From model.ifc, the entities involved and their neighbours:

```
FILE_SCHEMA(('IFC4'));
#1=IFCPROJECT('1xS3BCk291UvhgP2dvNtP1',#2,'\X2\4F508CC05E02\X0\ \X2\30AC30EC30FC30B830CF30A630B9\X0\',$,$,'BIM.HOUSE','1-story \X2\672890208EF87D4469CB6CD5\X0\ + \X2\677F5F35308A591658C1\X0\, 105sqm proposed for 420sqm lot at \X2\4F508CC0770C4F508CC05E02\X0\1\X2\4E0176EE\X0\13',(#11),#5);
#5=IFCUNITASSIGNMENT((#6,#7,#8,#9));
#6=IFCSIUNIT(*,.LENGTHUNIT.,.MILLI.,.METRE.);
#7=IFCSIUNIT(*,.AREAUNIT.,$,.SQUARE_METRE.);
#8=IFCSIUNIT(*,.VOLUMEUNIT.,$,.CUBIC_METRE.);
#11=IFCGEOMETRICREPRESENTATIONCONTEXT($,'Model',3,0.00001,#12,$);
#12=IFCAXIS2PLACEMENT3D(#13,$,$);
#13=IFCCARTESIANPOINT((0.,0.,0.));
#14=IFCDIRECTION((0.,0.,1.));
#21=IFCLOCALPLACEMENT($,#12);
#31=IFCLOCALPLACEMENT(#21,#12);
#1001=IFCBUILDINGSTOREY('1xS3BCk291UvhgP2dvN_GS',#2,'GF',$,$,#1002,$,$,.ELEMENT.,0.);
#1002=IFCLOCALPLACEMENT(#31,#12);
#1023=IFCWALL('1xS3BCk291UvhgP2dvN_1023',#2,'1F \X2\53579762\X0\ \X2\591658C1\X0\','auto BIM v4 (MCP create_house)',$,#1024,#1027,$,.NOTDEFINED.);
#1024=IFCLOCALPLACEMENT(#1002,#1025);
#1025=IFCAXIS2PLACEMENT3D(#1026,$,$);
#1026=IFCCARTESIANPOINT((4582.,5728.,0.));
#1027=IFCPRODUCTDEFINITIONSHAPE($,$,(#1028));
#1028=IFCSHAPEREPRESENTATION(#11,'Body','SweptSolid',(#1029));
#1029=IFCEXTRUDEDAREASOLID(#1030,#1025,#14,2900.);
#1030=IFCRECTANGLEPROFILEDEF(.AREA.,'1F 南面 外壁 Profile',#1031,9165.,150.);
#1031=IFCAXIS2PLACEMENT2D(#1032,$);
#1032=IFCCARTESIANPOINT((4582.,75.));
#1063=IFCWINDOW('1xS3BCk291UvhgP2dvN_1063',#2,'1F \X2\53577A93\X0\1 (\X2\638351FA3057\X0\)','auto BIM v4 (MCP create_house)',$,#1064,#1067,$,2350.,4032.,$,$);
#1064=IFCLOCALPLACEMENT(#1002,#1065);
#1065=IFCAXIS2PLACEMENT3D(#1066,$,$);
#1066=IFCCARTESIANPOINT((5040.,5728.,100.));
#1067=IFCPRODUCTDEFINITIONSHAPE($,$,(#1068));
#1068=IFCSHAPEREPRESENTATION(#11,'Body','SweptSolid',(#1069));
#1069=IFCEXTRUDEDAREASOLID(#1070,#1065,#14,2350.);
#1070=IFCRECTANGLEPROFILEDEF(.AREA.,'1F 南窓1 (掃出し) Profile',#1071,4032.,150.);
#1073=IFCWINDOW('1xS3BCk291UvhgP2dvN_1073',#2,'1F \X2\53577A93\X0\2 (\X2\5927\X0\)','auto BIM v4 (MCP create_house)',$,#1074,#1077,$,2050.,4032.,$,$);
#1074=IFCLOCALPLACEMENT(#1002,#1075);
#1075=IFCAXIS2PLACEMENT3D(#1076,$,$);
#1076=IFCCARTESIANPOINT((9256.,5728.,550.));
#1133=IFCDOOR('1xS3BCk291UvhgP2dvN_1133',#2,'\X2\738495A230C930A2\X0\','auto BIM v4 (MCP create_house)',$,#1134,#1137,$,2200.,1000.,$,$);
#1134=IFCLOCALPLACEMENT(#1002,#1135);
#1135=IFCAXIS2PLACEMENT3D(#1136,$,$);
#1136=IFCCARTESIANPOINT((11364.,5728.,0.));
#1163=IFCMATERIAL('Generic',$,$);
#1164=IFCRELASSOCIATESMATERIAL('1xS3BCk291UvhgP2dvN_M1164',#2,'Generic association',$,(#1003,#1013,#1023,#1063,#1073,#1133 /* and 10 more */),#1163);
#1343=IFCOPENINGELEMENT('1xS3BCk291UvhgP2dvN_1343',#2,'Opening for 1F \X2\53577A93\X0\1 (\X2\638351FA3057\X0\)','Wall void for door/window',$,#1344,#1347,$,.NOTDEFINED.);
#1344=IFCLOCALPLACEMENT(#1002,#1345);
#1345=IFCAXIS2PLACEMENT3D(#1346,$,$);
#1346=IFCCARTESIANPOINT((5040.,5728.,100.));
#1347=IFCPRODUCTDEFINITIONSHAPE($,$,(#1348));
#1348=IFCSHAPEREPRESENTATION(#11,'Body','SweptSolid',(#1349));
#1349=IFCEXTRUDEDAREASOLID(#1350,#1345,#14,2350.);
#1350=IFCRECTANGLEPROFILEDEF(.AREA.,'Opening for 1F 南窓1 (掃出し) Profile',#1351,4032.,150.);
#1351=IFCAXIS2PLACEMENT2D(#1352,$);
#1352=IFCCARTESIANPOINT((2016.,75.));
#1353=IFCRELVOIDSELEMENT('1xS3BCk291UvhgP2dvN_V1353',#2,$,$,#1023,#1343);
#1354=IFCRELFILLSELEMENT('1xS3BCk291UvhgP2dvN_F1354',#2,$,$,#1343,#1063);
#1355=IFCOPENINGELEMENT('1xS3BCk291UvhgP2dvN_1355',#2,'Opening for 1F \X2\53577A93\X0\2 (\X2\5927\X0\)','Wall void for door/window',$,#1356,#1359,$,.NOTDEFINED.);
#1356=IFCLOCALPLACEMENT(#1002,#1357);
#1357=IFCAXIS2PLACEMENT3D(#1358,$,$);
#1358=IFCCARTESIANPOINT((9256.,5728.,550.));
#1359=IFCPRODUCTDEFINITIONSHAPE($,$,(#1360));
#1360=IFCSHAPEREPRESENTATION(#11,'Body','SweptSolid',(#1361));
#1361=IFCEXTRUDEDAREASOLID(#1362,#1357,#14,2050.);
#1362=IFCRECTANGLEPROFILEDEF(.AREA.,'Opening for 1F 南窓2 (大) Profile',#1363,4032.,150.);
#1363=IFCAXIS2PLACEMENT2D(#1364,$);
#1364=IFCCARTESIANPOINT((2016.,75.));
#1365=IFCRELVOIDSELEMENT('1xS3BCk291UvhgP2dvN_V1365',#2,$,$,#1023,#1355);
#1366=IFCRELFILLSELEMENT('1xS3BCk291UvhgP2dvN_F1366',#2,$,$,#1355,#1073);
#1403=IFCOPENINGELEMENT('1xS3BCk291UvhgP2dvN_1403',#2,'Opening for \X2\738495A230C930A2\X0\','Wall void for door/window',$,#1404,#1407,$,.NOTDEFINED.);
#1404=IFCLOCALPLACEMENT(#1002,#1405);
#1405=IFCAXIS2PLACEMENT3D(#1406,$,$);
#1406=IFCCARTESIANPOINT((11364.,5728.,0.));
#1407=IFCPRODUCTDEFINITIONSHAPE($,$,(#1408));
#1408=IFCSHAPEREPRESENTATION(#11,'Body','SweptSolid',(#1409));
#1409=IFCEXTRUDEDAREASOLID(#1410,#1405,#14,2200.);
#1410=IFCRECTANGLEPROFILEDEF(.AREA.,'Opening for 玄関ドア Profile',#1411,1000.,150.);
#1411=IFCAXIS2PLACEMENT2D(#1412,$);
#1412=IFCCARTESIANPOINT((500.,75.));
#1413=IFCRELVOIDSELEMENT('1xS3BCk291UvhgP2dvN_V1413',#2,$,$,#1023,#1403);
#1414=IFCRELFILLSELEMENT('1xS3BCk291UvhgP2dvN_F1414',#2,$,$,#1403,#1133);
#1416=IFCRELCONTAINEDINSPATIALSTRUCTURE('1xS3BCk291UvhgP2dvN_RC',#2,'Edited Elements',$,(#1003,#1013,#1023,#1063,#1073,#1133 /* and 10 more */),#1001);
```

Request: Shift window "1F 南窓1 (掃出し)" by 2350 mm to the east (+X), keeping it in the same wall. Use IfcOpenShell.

```python
import ifcopenshell
import ifcopenshell.api.geometry
import ifcopenshell.util.placement
import ifcopenshell.util.unit

model = ifcopenshell.open("model.ifc")
unit_scale = ifcopenshell.util.unit.calculate_unit_scale(model)

window = model.by_guid("1xS3BCk291UvhgP2dvN_1063")
opening = window.FillsVoids[0].RelatingOpeningElement
wall = opening.VoidsElements[0].RelatingBuildingElement

wall_matrix = ifcopenshell.util.placement.get_local_placement(wall.ObjectPlacement)
shift = wall_matrix[:3, 0] * 2.35 / unit_scale
before = ifcopenshell.util.placement.get_local_placement(window.ObjectPlacement)[:3, 3].copy()

# The window is not placed relative to its opening, so move both.
for product in (opening, window):
    matrix = ifcopenshell.util.placement.get_local_placement(product.ObjectPlacement)
    matrix[:3, 3] += shift
    ifcopenshell.api.geometry.edit_object_placement(model, product=product, matrix=matrix, is_si=False)

after = ifcopenshell.util.placement.get_local_placement(window.ObjectPlacement)[:3, 3]
print("window moved by", (after - before).round(3) + 0.0)

model.write("model-out.ifc")
```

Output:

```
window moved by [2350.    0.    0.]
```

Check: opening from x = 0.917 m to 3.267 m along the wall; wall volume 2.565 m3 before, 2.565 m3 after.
